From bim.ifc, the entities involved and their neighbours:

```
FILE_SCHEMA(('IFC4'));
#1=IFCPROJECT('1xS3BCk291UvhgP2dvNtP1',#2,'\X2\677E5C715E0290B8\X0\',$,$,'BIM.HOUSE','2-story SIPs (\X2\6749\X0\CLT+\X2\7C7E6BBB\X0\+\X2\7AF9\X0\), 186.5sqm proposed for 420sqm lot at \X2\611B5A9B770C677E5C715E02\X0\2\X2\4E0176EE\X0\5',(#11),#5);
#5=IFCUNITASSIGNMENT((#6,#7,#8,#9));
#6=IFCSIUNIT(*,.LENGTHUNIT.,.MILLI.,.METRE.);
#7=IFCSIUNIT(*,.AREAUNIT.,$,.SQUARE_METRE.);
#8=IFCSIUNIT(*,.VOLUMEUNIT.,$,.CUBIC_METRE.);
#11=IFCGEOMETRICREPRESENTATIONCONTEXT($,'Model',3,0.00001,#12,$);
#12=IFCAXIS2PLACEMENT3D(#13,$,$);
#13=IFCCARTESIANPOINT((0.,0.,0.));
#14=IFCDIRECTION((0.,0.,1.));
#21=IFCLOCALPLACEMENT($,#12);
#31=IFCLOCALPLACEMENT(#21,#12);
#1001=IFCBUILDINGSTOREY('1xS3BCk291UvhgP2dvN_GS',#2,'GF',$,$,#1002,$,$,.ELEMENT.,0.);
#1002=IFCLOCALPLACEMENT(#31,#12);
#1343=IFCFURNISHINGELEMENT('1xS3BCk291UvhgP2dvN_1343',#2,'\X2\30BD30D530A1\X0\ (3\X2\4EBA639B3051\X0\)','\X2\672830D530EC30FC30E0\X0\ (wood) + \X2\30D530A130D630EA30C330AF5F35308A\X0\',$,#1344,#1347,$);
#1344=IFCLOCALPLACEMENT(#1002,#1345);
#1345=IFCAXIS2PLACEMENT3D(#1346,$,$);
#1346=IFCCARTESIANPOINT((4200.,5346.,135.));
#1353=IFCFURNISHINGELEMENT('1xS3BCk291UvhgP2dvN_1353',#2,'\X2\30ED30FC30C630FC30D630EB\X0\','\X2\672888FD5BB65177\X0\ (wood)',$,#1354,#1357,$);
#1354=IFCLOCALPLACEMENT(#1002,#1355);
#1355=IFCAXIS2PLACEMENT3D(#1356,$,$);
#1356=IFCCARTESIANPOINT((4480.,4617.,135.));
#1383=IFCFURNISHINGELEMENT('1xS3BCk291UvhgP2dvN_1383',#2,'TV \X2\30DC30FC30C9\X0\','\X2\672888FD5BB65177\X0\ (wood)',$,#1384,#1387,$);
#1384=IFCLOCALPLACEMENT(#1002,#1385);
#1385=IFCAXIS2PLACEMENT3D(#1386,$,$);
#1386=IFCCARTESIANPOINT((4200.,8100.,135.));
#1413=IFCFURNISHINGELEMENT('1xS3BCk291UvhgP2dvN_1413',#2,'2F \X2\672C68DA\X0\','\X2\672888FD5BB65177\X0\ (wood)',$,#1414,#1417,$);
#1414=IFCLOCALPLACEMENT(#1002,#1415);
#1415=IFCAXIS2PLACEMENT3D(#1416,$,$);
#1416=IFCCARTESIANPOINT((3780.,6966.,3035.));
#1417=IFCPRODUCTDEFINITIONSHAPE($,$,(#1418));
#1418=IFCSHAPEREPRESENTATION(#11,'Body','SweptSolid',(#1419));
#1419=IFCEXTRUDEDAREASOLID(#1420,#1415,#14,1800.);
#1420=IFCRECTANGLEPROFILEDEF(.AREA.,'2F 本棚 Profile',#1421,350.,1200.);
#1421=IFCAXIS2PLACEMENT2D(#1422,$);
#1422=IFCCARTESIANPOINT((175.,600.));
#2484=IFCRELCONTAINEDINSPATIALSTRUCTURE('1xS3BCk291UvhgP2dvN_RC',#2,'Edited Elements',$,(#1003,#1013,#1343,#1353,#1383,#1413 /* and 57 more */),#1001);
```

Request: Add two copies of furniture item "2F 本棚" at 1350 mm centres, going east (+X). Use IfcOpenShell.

```python
import numpy as np
import ifcopenshell
import ifcopenshell.api.geometry
import ifcopenshell.api.root
import ifcopenshell.util.element
import ifcopenshell.util.placement

model = ifcopenshell.open("bim.ifc")


def reuse_history(source, copy):
    """copy_class also copies each property set's owner history, people and application; keep the originals."""
    for rel in copy.IsDefinedBy:
        if rel.is_a("IfcRelDefinesByProperties") and (history := rel.RelatingPropertyDefinition.OwnerHistory):
            rel.RelatingPropertyDefinition.OwnerHistory = source.OwnerHistory
            ifcopenshell.util.element.remove_deep2(model, history)


source = model.by_id(1413)
base = ifcopenshell.util.placement.get_local_placement(source.ObjectPlacement)
step = np.array([1.0, 0.0, 0.0]) * 1350.0

for i in range(1, 3):
    copy = ifcopenshell.api.root.copy_class(model, product=source)
    copy.Representation = ifcopenshell.util.element.copy_deep(
        model, source.Representation, exclude=["IfcGeometricRepresentationContext", "IfcRepresentationMap"]
    )
    reuse_history(source, copy)
    matrix = base.copy()
    matrix[:3, 3] += i * step
    print("added at", matrix[:3, 3].round(3) + 0.0)
    ifcopenshell.api.geometry.edit_object_placement(model, product=copy, matrix=matrix, is_si=False)

model.write("bim_v2.ifc")
```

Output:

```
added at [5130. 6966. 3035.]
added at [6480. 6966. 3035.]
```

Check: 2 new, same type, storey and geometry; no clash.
